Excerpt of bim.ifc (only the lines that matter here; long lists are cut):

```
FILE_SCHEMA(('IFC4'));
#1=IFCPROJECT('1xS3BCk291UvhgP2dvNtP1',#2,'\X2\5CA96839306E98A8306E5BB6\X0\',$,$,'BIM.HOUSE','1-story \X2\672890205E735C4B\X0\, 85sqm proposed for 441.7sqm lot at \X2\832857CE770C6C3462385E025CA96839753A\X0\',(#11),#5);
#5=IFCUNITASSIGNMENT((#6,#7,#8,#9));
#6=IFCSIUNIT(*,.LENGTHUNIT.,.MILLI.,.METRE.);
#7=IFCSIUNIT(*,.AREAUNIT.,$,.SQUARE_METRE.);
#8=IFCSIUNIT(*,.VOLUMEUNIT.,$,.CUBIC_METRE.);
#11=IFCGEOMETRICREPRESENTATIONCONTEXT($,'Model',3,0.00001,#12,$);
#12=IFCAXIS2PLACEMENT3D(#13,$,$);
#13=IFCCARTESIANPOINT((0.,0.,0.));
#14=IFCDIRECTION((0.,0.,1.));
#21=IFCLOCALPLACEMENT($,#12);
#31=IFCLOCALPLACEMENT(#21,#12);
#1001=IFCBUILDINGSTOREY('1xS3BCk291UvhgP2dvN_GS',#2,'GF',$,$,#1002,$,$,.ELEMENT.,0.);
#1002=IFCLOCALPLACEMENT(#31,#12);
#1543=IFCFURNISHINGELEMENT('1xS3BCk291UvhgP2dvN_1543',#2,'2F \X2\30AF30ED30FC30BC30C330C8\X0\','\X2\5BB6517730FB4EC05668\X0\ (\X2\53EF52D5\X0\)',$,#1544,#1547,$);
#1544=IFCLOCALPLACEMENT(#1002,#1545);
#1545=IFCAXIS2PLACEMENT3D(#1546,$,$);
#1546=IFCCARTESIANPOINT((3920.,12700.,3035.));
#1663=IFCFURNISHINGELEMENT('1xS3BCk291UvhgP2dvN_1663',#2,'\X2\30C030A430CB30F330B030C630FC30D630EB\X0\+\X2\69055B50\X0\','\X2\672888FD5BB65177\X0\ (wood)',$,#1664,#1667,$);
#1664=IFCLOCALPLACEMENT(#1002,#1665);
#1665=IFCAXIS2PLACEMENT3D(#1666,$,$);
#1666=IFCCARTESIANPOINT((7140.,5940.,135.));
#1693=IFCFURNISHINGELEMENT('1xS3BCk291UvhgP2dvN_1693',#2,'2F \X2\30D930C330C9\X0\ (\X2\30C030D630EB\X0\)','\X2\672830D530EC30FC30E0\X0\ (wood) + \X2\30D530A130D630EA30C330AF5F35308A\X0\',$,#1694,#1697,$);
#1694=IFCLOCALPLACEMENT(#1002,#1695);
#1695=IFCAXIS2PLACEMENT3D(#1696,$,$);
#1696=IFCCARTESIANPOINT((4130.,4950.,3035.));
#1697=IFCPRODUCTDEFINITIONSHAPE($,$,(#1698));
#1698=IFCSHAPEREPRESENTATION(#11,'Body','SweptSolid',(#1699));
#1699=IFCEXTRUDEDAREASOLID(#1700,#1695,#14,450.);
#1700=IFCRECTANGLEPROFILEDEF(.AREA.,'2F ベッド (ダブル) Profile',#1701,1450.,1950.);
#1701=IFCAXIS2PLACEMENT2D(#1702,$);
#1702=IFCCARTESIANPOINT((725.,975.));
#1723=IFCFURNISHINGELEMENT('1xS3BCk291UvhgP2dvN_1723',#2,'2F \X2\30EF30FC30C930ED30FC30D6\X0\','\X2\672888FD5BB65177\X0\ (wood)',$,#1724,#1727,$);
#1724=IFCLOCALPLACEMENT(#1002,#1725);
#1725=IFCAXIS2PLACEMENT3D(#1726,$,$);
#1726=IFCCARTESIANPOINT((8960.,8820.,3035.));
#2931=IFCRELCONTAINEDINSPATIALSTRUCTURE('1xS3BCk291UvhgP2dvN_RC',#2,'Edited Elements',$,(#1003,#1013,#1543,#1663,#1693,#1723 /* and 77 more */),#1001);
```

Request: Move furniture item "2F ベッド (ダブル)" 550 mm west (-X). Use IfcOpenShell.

```python
import ifcopenshell
import ifcopenshell.api.geometry
import ifcopenshell.util.placement
import ifcopenshell.util.unit

model = ifcopenshell.open("bim.ifc")
unit_scale = ifcopenshell.util.unit.calculate_unit_scale(model)

item = model.by_guid("1xS3BCk291UvhgP2dvN_1693")
matrix = ifcopenshell.util.placement.get_local_placement(item.ObjectPlacement)
matrix[0, 3] -= 0.55 / unit_scale
ifcopenshell.api.geometry.edit_object_placement(model, product=item, matrix=matrix, is_si=False)

print(ifcopenshell.util.placement.get_local_placement(item.ObjectPlacement).round(3) + 0.0)

model.write("bim_edited.ifc")
```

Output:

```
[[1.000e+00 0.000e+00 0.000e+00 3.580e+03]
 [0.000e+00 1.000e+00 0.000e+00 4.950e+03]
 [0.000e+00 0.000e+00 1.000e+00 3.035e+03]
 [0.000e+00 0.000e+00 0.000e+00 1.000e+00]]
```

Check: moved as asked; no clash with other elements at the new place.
